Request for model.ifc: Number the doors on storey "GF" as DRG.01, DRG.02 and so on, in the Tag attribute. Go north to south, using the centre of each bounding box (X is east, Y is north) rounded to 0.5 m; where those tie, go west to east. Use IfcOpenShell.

First a look at what the model holds.

```python
import ifcopenshell
import ifcopenshell.util.element
import ifcopenshell.util.placement

model = ifcopenshell.open("model.ifc")
print(model.schema)
storey = next(s for s in model.by_type("IfcBuildingStorey") if s.Name == "GF")
doors = [e for e in ifcopenshell.util.element.get_decomposition(storey) if e.is_a("IfcDoor")]
for e in sorted(doors, key=lambda e: e.id()):
    origin = ifcopenshell.util.placement.get_local_placement(e.ObjectPlacement)[:3, 3]
    print(e.id(), e.Tag, e.Name, origin.round(2) + 0.0, sep=" | ")
```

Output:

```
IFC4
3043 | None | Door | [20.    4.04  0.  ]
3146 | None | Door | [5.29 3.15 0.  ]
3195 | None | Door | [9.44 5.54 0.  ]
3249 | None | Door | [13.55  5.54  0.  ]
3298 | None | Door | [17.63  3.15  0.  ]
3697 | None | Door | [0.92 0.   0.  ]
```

```python
import ifcopenshell
import ifcopenshell.geom
import ifcopenshell.util.element
import ifcopenshell.util.shape

model = ifcopenshell.open("model.ifc")
settings = ifcopenshell.geom.settings()
settings.set("use-world-coords", True)


def centre(element):
    shape = ifcopenshell.geom.create_shape(settings, element)
    return ifcopenshell.util.shape.get_bbox_centroid(shape.geometry)


storey = next(s for s in model.by_type("IfcBuildingStorey") if s.Name == "GF")
doors = [e for e in ifcopenshell.util.element.get_decomposition(storey) if e.is_a("IfcDoor")]

# Insertion points can sit at a corner or the storey origin, so sort by the geometry (in metres).
centres = {e: centre(e) for e in doors}
doors.sort(key=lambda e: (-round(centres[e][1] / 0.5), centres[e][0]))

for i, e in enumerate(doors, start=1):
    number = f"DRG.{i:02d}"
    e.Tag = number
    print(e.id(), number)

model.write("model_updated.ifc")
```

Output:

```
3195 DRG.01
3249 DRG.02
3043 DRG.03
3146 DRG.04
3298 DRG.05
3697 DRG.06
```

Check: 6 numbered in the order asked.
